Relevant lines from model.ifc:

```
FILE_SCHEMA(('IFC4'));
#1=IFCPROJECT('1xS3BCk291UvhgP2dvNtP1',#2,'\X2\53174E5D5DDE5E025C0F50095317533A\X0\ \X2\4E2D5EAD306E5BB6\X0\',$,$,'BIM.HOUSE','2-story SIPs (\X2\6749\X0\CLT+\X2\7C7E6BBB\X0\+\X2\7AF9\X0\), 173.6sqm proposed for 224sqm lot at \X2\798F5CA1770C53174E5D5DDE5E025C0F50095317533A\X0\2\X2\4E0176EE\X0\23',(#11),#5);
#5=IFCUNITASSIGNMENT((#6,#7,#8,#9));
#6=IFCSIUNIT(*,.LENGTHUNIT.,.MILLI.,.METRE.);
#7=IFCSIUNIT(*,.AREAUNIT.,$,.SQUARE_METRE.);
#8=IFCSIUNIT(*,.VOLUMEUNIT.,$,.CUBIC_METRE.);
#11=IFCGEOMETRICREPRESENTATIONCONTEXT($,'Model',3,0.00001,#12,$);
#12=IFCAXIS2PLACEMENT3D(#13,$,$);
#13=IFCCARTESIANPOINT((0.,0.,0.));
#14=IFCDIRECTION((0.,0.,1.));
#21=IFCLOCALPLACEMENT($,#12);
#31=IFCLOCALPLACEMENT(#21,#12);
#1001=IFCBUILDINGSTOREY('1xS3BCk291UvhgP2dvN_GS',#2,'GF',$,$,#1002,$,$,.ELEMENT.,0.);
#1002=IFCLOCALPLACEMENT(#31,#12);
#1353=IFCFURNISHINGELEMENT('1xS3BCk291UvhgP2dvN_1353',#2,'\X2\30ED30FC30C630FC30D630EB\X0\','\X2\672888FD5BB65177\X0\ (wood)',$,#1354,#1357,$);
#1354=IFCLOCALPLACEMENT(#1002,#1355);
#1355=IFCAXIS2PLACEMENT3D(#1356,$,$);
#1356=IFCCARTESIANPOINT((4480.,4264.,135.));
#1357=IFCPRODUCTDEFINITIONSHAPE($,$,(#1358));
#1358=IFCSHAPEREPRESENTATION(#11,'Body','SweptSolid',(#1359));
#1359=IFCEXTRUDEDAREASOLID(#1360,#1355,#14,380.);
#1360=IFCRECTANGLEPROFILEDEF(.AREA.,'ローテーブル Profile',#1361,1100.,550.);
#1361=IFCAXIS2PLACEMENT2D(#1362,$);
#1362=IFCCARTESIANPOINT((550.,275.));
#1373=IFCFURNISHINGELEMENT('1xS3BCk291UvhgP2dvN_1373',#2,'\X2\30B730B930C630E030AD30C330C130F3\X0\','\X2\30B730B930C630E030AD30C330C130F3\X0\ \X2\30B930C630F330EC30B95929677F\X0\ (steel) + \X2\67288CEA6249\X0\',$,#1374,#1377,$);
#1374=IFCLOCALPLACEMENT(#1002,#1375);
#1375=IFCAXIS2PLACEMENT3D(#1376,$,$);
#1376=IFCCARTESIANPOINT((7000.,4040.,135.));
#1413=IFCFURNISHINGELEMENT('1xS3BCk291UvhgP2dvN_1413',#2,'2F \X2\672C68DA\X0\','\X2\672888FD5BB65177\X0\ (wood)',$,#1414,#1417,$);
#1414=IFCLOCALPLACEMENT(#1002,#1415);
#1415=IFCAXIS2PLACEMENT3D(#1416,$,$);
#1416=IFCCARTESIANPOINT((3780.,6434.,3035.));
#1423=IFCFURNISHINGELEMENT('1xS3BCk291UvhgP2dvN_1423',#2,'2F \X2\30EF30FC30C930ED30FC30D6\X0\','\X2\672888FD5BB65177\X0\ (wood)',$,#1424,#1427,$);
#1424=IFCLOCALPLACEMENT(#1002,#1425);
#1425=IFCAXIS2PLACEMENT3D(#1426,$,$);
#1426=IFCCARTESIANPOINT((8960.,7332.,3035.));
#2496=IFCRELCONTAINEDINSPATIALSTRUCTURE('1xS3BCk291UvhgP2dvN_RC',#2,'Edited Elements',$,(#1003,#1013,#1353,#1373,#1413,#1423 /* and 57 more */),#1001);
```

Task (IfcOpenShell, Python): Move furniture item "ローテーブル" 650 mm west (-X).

```python
import ifcopenshell
import ifcopenshell.api.geometry
import ifcopenshell.util.placement

model = ifcopenshell.open("model.ifc")

item = model.by_guid("1xS3BCk291UvhgP2dvN_1353")
matrix = ifcopenshell.util.placement.get_local_placement(item.ObjectPlacement)
matrix[0, 3] -= 650.0
ifcopenshell.api.geometry.edit_object_placement(model, product=item, matrix=matrix, is_si=False)

print(ifcopenshell.util.placement.get_local_placement(item.ObjectPlacement).round(3) + 0.0)

model.write("model_rev.ifc")
```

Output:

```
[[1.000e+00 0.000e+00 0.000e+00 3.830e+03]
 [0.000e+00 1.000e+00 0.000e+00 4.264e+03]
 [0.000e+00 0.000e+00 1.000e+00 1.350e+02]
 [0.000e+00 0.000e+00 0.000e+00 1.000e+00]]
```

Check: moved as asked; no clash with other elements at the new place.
